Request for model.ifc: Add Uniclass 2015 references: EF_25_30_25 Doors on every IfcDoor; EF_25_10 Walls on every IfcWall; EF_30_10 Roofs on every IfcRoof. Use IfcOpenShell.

First a look at what the model holds.

```python
import ifcopenshell

model = ifcopenshell.open("model.ifc")
print(model.schema)
print("classifications:", [c.Name for c in model.by_type("IfcClassification")])
for ifc_class in ("IfcDoor", "IfcRoof", "IfcStair", "IfcWall", "IfcWindow"):
    print(ifc_class, len(model.by_type(ifc_class)))
```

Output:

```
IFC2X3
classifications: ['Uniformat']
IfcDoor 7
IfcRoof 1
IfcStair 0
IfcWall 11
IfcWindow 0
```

```python
import ifcopenshell
import ifcopenshell.api.classification

model = ifcopenshell.open("model.ifc")

# IFC2X3 requires Source and Edition and has no link from the project to the system.
system = model.create_entity("IfcClassification", Source="NBS", Edition="2015", Name="Uniclass 2015")

codes = {
    "IfcDoor": ("EF_25_30_25", "Doors"),
    "IfcWall": ("EF_25_10", "Walls"),
    "IfcRoof": ("EF_30_10", "Roofs"),
}
for ifc_class, (code, name) in codes.items():
    products = model.by_type(ifc_class)
    ifcopenshell.api.classification.add_reference(
        model, products=products, classification=system, identification=code, name=name
    )
    print(code, len(products))

model.write("model_v2.ifc")
```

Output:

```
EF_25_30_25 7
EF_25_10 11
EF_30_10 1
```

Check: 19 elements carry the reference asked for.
